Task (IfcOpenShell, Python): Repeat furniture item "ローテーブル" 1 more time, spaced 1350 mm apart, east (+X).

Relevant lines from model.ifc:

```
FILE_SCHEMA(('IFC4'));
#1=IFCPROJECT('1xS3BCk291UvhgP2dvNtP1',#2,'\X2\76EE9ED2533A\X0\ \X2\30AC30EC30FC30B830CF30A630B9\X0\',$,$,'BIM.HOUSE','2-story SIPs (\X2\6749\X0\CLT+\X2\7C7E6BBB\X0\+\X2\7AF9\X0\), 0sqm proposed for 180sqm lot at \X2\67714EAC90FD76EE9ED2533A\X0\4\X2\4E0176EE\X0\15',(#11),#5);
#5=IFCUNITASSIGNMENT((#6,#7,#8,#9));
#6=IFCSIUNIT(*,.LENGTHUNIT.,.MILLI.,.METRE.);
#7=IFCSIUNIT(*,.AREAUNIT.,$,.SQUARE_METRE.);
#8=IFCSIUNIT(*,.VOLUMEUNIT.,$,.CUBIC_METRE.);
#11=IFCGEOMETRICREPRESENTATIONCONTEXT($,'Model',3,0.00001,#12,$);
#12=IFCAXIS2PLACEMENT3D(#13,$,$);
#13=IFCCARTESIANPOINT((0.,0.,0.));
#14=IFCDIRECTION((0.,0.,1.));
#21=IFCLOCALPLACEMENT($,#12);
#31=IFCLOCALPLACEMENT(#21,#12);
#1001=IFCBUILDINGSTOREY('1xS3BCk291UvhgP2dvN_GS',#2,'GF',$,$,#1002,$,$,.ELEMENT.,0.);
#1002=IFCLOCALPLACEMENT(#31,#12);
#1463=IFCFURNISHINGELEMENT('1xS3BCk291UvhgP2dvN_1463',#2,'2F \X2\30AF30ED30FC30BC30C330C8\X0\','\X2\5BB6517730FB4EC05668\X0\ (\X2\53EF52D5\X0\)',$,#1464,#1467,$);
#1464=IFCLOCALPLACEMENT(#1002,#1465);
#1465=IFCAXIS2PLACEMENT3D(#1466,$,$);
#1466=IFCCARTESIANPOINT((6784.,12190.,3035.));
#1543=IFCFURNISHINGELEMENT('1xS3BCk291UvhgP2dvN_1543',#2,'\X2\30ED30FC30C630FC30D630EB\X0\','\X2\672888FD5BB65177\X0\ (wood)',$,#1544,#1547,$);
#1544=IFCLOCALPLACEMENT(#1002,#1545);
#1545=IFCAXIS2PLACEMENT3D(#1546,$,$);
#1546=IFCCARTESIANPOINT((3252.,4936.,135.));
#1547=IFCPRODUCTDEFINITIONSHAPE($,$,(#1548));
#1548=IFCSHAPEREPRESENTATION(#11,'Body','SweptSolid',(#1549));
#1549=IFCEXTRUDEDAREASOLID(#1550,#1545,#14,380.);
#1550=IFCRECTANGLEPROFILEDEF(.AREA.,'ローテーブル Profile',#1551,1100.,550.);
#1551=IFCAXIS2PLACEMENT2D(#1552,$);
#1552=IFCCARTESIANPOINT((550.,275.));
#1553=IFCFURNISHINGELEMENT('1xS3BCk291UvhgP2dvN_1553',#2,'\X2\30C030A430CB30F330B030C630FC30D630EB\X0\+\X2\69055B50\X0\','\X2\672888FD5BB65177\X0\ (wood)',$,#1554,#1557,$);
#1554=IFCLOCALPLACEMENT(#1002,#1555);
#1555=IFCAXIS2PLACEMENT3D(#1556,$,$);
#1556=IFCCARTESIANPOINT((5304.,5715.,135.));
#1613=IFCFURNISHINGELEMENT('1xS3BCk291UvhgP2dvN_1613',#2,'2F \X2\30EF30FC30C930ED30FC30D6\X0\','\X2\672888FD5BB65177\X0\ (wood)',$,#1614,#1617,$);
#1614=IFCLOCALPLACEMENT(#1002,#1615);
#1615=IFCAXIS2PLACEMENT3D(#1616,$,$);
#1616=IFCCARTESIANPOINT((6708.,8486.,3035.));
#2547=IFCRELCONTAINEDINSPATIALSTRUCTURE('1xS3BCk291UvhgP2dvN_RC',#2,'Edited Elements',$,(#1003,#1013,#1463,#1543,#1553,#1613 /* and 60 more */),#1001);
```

```python
import numpy as np
import ifcopenshell
import ifcopenshell.api.geometry
import ifcopenshell.api.root
import ifcopenshell.util.element
import ifcopenshell.util.placement
import ifcopenshell.util.unit

model = ifcopenshell.open("model.ifc")
unit_scale = ifcopenshell.util.unit.calculate_unit_scale(model)


def reuse_history(source, copy):
    """copy_class also copies each property set's owner history, people and application; keep the originals."""
    for rel in copy.IsDefinedBy:
        if rel.is_a("IfcRelDefinesByProperties") and (history := rel.RelatingPropertyDefinition.OwnerHistory):
            rel.RelatingPropertyDefinition.OwnerHistory = source.OwnerHistory
            ifcopenshell.util.element.remove_deep2(model, history)


source = model.by_guid("1xS3BCk291UvhgP2dvN_1543")
base = ifcopenshell.util.placement.get_local_placement(source.ObjectPlacement)
step = np.array([1.0, 0.0, 0.0]) * 1.35 / unit_scale

for i in range(1, 2):
    copy = ifcopenshell.api.root.copy_class(model, product=source)
    copy.Representation = ifcopenshell.util.element.copy_deep(
        model, source.Representation, exclude=["IfcGeometricRepresentationContext", "IfcRepresentationMap"]
    )
    reuse_history(source, copy)
    matrix = base.copy()
    matrix[:3, 3] += i * step
    print("added at", matrix[:3, 3].round(3) + 0.0)
    ifcopenshell.api.geometry.edit_object_placement(model, product=copy, matrix=matrix, is_si=False)

model.write("model_updated.ifc")
```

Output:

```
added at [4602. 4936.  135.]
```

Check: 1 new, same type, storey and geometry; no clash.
